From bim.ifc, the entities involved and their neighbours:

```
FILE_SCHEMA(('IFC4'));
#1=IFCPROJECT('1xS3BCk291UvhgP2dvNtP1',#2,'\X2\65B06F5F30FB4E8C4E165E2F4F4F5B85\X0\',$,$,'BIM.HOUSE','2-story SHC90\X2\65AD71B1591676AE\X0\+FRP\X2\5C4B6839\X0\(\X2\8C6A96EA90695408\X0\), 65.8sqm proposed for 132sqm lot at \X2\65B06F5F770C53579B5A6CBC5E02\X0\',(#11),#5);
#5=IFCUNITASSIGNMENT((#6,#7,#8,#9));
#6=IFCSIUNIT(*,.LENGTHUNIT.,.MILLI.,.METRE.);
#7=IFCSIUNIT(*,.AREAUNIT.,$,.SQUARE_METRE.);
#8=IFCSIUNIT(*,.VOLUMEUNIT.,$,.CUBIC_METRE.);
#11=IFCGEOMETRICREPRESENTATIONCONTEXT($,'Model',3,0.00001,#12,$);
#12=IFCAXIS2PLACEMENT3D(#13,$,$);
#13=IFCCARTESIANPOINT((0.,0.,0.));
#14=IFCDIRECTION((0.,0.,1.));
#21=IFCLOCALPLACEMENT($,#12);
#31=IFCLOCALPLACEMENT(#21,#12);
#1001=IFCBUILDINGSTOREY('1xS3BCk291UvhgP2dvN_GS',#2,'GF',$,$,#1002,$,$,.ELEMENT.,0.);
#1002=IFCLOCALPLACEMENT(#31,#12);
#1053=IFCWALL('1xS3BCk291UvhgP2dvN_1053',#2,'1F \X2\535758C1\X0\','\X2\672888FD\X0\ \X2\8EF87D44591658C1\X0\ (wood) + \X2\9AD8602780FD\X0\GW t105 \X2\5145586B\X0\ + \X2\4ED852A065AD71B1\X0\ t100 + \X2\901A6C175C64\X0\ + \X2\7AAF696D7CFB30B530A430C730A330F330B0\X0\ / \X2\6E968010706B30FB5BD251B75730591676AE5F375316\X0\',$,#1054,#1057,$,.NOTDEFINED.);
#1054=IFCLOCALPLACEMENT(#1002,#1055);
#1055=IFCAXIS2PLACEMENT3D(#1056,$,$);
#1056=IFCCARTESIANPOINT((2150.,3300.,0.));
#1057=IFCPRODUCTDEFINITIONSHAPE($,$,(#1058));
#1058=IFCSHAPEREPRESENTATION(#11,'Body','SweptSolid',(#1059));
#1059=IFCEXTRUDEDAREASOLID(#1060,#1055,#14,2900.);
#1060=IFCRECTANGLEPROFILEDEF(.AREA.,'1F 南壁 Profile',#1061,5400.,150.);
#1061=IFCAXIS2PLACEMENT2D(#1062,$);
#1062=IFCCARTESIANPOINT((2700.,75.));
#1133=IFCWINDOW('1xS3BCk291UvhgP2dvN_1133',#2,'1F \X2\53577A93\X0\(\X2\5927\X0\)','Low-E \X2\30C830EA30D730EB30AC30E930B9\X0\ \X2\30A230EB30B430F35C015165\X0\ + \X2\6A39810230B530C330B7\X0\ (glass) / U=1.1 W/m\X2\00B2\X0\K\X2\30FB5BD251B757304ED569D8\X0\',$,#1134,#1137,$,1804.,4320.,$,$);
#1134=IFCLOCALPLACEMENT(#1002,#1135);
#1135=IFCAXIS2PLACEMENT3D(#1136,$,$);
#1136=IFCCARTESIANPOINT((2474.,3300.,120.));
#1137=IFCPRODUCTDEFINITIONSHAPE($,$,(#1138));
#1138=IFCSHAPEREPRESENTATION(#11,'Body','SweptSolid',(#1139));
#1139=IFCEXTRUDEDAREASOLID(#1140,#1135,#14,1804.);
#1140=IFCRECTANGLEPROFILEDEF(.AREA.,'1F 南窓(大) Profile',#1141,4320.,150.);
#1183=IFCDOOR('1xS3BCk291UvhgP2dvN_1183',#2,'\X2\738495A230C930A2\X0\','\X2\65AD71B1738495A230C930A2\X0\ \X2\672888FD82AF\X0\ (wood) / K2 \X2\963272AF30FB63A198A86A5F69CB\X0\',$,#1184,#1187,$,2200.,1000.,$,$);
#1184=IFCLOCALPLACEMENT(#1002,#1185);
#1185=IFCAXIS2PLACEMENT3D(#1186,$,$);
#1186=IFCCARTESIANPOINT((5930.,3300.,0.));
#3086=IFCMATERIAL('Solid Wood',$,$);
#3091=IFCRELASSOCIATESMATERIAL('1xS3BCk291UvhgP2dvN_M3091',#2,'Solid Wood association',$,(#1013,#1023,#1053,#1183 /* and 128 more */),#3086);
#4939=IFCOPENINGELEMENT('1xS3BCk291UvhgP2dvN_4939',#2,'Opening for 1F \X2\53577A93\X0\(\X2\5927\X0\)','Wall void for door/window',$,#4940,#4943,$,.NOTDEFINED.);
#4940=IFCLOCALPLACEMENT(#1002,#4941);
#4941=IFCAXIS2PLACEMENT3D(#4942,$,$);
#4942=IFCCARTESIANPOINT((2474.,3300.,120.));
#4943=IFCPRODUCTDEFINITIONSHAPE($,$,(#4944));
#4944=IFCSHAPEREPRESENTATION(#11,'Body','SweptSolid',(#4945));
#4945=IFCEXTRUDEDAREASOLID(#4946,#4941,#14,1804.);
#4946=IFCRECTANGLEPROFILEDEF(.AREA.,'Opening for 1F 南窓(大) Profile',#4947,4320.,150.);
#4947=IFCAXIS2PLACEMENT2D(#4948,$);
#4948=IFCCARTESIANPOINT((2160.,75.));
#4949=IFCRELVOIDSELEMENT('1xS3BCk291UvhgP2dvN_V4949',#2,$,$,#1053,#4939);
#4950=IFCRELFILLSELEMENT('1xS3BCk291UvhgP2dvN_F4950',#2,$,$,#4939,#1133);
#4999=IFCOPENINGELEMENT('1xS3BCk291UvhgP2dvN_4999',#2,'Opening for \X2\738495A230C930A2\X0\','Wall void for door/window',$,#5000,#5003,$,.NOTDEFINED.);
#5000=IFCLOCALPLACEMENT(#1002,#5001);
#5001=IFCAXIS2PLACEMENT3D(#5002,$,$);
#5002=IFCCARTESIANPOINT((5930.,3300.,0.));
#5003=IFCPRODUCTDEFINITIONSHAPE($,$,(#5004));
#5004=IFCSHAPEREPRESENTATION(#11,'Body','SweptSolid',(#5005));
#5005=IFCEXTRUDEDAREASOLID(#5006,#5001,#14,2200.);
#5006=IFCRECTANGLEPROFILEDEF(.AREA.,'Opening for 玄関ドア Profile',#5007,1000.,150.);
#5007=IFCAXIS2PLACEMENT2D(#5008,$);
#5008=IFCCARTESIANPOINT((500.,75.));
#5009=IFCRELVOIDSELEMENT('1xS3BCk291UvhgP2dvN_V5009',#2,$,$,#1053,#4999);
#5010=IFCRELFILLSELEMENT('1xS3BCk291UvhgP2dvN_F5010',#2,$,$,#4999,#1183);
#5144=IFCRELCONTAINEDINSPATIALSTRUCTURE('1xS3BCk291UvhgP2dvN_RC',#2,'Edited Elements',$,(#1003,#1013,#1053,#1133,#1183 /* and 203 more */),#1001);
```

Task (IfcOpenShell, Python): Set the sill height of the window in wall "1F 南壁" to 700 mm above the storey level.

```python
import numpy as np
import ifcopenshell
import ifcopenshell.api.geometry
import ifcopenshell.geom
import ifcopenshell.util.element
import ifcopenshell.util.placement
import ifcopenshell.util.shape
import ifcopenshell.util.unit

model = ifcopenshell.open("bim.ifc")
unit_scale = ifcopenshell.util.unit.calculate_unit_scale(model)

window = model.by_guid("1xS3BCk291UvhgP2dvN_1133")
opening = window.FillsVoids[0].RelatingOpeningElement
storey = ifcopenshell.util.element.get_container(window, ifc_class="IfcBuildingStorey")
level = ifcopenshell.util.placement.get_local_placement(storey.ObjectPlacement)[2, 3]

# The opening's origin need not be at the sill, so measure its lowest point.
shape = ifcopenshell.geom.create_shape(ifcopenshell.geom.settings(), opening)
bottom = ifcopenshell.util.shape.get_shape_bottom_elevation(shape, shape.geometry) / unit_scale
dz = level + 700.0 - bottom

shift = np.array([0.0, 0.0, dz])
# The window is not placed relative to its opening, so move both.
for product in (opening, window):
    matrix = ifcopenshell.util.placement.get_local_placement(product.ObjectPlacement)
    matrix[:3, 3] += shift
    ifcopenshell.api.geometry.edit_object_placement(model, product=product, matrix=matrix, is_si=False)

print(f"moved by {dz * unit_scale:+.3f} m")

model.write("bim_v2.ifc")
```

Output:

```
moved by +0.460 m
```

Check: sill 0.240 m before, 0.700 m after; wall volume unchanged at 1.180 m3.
